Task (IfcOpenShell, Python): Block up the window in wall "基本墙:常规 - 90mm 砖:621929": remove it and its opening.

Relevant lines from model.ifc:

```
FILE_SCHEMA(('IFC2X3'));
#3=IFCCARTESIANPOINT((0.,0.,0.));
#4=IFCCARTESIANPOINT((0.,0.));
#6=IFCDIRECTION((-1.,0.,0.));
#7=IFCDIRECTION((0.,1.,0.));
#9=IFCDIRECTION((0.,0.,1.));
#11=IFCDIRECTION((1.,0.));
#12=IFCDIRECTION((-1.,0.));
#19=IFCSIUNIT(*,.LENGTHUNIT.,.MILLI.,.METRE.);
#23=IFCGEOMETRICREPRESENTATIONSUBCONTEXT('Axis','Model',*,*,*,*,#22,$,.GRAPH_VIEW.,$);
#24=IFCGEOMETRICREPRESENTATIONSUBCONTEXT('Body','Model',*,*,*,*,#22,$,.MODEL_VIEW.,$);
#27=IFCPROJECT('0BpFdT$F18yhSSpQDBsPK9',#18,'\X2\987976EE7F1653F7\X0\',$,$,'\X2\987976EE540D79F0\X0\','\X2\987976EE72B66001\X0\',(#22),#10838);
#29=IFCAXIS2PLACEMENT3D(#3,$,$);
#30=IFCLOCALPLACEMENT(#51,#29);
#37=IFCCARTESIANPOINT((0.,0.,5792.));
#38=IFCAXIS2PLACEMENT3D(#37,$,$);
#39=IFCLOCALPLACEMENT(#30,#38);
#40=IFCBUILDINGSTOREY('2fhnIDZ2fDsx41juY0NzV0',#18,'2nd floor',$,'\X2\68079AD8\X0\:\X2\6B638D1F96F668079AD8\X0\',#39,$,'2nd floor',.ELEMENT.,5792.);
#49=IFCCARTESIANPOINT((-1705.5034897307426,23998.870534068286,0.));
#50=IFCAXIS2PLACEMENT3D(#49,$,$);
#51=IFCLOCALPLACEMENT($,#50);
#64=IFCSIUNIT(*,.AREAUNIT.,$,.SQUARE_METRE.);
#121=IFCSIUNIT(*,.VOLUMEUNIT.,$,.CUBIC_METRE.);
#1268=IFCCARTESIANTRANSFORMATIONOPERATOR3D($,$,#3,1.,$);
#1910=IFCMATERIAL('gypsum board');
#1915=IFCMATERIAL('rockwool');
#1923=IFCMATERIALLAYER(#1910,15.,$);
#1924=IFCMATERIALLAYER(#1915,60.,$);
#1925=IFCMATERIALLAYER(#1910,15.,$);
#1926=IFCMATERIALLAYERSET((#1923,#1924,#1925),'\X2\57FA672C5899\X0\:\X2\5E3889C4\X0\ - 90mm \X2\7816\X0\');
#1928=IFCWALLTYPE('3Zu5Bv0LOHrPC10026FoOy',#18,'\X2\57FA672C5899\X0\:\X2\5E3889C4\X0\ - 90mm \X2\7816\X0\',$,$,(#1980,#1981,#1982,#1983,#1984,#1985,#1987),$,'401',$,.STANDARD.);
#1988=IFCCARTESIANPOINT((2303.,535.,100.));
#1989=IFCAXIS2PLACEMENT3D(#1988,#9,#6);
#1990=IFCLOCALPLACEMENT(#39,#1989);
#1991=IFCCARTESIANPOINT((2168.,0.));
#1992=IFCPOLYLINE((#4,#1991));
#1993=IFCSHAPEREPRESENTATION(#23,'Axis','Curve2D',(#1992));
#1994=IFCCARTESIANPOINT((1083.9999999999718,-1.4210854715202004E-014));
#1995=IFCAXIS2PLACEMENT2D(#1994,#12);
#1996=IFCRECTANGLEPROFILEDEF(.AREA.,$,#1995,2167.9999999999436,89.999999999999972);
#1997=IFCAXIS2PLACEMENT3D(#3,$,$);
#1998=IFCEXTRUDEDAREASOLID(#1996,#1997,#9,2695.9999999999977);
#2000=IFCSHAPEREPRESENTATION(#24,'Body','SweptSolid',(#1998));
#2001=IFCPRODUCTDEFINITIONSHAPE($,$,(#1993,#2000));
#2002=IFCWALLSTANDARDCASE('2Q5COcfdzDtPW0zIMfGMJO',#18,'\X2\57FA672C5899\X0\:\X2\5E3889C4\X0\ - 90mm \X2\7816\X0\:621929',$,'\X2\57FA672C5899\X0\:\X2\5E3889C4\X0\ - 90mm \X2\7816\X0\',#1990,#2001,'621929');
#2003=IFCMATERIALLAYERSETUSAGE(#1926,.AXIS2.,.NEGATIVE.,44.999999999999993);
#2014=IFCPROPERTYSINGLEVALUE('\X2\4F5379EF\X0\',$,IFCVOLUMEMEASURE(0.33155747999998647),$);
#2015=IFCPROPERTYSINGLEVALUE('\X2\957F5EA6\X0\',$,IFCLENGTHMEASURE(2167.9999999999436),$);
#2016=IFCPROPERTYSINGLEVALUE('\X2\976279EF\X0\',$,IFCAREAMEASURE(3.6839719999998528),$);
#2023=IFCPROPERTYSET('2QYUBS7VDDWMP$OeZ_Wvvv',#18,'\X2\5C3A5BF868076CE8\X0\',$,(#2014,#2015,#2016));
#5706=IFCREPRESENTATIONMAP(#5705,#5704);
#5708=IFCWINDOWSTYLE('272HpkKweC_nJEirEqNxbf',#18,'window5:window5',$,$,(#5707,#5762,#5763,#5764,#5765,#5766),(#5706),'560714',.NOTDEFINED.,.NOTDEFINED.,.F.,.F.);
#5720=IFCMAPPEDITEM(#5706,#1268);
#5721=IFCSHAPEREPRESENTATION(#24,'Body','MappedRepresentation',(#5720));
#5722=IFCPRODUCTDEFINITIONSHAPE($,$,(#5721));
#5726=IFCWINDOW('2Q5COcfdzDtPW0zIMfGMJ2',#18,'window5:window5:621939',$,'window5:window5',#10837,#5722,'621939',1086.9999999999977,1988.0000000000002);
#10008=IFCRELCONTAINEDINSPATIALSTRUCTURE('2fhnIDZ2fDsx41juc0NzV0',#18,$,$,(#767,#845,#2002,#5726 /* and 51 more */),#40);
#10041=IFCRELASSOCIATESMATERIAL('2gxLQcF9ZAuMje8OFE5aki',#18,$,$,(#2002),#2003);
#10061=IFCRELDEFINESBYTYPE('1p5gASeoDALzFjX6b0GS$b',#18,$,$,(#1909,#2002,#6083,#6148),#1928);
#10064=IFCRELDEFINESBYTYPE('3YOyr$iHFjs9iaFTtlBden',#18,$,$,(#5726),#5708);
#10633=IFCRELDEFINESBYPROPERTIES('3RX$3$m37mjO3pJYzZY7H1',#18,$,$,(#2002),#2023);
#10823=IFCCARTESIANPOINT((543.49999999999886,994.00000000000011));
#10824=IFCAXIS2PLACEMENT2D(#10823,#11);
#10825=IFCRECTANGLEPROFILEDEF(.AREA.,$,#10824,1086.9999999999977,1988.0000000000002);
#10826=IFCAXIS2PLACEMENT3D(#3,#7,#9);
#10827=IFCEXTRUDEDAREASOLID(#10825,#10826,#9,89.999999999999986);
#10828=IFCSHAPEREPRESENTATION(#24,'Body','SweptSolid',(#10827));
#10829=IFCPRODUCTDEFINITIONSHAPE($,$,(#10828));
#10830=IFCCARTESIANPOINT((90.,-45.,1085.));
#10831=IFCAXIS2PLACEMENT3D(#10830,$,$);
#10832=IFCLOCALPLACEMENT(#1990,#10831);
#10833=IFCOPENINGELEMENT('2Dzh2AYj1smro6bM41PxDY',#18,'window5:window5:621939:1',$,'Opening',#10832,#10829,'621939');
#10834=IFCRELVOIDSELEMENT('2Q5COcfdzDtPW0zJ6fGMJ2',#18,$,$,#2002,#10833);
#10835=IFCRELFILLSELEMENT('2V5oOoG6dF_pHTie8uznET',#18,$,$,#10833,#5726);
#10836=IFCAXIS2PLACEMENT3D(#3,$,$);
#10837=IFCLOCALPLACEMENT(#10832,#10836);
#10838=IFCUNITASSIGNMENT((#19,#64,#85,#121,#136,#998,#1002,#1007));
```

```python
import ifcopenshell
import ifcopenshell.api.feature
import ifcopenshell.api.pset
import ifcopenshell.api.root
import ifcopenshell.geom
import ifcopenshell.util.element
import ifcopenshell.util.shape
import ifcopenshell.util.unit

model = ifcopenshell.open("model.ifc")
area_scale = ifcopenshell.util.unit.calculate_unit_scale(model, "AREAUNIT")
volume_scale = ifcopenshell.util.unit.calculate_unit_scale(model, "VOLUMEUNIT")
settings = ifcopenshell.geom.settings()


def volume(element):
    """Net volume in cubic metres, openings subtracted."""
    shape = ifcopenshell.geom.create_shape(settings, element)
    return ifcopenshell.util.shape.get_volume(shape.geometry)


window = model.by_guid("2Q5COcfdzDtPW0zIMfGMJ2")
opening = window.FillsVoids[0].RelatingOpeningElement
wall = opening.VoidsElements[0].RelatingBuildingElement
before = volume(wall)

ifcopenshell.api.root.remove_product(model, product=window)
ifcopenshell.api.feature.remove_feature(model, feature=opening)

after = volume(wall)
thickness = 0.09  # wall thickness in metres

# Update the wall's stored quantities.
pset = model.by_id(ifcopenshell.util.element.get_pset(wall, "尺寸标注", should_inherit=False)["id"])
ifcopenshell.api.pset.edit_pset(model, pset=pset, properties={
    "体积": model.create_entity("IfcVolumeMeasure", after / volume_scale),
    "面积": model.create_entity("IfcAreaMeasure", after / thickness / area_scale),
})

print(f"wall volume {before:.3f} -> {after:.3f} m3")

model.write("model_v2.ifc")
```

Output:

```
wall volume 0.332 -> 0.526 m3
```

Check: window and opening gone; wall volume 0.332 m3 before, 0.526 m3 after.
